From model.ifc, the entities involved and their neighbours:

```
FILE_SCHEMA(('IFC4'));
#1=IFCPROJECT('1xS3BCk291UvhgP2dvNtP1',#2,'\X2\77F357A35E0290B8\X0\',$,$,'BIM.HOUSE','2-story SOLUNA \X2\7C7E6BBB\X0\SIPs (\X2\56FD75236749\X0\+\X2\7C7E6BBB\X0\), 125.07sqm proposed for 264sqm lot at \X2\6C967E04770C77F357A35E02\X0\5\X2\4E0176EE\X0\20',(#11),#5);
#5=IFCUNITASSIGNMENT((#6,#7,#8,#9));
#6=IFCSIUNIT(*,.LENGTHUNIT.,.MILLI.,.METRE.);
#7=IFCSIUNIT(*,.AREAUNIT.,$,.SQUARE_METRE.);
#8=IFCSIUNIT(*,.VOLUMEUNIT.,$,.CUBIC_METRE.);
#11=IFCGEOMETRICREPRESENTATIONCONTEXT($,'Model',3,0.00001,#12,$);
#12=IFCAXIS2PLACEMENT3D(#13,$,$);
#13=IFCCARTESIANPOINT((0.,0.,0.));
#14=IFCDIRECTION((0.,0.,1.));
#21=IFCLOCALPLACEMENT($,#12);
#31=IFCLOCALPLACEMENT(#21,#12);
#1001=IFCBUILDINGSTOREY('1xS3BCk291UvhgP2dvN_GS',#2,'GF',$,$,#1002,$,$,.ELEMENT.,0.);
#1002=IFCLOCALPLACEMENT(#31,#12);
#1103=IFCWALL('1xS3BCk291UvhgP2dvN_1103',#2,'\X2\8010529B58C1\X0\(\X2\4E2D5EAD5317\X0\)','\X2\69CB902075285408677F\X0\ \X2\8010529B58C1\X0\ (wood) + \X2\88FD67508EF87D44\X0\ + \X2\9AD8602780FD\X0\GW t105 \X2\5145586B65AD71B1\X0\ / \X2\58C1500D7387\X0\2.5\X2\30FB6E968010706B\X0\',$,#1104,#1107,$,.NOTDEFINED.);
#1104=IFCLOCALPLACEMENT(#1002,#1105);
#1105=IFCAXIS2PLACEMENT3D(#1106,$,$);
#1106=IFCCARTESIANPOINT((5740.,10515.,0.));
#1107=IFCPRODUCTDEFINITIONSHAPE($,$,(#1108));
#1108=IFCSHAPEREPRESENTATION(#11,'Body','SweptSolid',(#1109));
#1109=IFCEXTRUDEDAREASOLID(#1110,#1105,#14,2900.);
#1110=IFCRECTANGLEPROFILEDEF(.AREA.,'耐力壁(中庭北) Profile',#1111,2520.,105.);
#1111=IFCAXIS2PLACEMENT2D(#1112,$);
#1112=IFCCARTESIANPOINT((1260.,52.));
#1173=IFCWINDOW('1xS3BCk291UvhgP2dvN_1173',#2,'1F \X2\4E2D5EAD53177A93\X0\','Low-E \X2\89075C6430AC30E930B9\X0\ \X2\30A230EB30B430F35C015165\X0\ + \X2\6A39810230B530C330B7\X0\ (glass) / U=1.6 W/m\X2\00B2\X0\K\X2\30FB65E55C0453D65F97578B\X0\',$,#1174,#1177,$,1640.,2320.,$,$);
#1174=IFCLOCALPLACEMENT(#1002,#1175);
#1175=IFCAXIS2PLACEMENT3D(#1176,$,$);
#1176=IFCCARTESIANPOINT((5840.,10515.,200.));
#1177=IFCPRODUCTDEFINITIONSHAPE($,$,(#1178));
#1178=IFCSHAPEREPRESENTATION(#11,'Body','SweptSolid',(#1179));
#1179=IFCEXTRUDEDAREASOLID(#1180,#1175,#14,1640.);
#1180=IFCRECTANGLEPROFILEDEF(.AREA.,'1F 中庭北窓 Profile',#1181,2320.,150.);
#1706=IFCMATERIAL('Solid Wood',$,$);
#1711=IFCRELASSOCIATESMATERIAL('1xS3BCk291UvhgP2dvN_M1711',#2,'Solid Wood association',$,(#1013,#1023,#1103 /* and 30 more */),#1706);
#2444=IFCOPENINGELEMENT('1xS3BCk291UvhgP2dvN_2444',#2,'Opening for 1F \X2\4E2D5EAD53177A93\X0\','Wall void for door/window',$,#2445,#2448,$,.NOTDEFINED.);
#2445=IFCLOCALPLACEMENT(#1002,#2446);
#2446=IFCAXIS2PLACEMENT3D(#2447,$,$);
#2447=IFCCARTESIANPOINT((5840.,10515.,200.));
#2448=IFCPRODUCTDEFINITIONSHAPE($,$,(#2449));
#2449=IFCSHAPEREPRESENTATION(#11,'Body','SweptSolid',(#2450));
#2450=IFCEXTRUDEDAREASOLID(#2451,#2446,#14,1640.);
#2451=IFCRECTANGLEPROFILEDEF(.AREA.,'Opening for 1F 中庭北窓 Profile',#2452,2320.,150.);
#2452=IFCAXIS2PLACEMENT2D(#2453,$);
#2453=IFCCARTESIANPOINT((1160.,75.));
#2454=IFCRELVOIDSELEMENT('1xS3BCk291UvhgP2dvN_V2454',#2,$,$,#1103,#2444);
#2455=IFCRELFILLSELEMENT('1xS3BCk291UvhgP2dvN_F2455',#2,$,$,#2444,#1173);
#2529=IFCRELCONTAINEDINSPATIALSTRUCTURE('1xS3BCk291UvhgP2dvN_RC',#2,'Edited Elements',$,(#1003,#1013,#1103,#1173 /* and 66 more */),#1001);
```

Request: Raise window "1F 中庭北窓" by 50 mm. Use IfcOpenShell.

```python
import numpy as np
import ifcopenshell
import ifcopenshell.api.geometry
import ifcopenshell.util.placement
import ifcopenshell.util.unit

model = ifcopenshell.open("model.ifc")
unit_scale = ifcopenshell.util.unit.calculate_unit_scale(model)

window = model.by_guid("1xS3BCk291UvhgP2dvN_1173")
opening = window.FillsVoids[0].RelatingOpeningElement
dz = 0.05 / unit_scale

shift = np.array([0.0, 0.0, dz])
# The window is not placed relative to its opening, so move both.
for product in (opening, window):
    matrix = ifcopenshell.util.placement.get_local_placement(product.ObjectPlacement)
    matrix[:3, 3] += shift
    ifcopenshell.api.geometry.edit_object_placement(model, product=product, matrix=matrix, is_si=False)

print(f"moved by {dz * unit_scale:+.3f} m")

model.write("model_updated.ifc")
```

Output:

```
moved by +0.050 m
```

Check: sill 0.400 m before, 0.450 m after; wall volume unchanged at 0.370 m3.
